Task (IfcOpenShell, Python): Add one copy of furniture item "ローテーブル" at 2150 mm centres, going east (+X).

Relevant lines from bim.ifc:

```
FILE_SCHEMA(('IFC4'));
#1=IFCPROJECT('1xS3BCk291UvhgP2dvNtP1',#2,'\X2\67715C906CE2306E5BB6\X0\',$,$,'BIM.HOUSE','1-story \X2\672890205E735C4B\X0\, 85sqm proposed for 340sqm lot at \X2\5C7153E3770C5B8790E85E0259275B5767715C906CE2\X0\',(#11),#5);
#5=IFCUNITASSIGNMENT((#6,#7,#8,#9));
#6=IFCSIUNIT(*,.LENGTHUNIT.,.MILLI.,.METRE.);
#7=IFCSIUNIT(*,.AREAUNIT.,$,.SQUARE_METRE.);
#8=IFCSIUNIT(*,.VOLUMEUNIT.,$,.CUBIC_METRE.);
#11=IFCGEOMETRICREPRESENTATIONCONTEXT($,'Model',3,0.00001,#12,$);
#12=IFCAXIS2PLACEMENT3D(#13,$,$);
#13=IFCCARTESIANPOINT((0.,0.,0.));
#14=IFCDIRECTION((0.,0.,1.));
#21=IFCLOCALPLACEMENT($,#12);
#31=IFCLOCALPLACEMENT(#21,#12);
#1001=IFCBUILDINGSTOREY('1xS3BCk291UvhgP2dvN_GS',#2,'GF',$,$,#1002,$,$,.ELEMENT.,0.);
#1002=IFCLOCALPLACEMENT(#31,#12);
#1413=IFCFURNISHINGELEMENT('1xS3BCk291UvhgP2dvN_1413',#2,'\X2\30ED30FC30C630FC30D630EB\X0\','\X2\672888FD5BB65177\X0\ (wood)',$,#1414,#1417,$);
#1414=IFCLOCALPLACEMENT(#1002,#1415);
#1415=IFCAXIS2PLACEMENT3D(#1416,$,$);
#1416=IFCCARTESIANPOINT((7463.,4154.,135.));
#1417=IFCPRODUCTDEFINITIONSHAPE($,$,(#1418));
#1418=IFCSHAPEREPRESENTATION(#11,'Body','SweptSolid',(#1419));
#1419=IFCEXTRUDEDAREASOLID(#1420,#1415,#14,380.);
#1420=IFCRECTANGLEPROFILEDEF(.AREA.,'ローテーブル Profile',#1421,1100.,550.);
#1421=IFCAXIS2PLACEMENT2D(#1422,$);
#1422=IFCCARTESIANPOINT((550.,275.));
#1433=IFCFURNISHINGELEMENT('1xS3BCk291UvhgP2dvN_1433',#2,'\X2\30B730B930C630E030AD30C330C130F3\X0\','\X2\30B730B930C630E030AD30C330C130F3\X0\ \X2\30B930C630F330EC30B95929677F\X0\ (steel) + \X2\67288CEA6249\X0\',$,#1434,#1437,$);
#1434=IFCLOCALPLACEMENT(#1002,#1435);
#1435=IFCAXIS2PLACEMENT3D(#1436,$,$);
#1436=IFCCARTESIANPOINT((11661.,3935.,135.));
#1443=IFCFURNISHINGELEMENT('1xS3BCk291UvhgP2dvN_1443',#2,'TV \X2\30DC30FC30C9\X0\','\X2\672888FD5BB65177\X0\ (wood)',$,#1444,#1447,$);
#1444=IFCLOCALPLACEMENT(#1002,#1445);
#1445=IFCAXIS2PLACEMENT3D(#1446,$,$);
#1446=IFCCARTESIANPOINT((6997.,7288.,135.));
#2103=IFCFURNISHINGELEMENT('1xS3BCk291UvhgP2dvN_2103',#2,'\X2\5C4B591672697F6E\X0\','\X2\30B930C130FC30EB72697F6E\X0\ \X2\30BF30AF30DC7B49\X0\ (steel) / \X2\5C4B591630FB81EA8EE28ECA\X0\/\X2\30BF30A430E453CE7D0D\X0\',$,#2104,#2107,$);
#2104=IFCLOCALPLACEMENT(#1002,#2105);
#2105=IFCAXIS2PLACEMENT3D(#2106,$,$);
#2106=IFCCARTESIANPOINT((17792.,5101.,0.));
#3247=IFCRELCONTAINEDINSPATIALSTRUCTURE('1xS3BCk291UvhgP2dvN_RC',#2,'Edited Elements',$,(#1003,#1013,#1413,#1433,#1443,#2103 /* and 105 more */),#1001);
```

```python
import numpy as np
import ifcopenshell
import ifcopenshell.api.geometry
import ifcopenshell.api.root
import ifcopenshell.util.element
import ifcopenshell.util.placement

model = ifcopenshell.open("bim.ifc")


def reuse_history(source, copy):
    """copy_class also copies each property set's owner history, people and application; keep the originals."""
    for rel in copy.IsDefinedBy:
        if rel.is_a("IfcRelDefinesByProperties") and (history := rel.RelatingPropertyDefinition.OwnerHistory):
            rel.RelatingPropertyDefinition.OwnerHistory = source.OwnerHistory
            ifcopenshell.util.element.remove_deep2(model, history)


source = model.by_guid("1xS3BCk291UvhgP2dvN_1413")
base = ifcopenshell.util.placement.get_local_placement(source.ObjectPlacement)
step = np.array([1.0, 0.0, 0.0]) * 2150.0

for i in range(1, 2):
    copy = ifcopenshell.api.root.copy_class(model, product=source)
    copy.Representation = ifcopenshell.util.element.copy_deep(
        model, source.Representation, exclude=["IfcGeometricRepresentationContext", "IfcRepresentationMap"]
    )
    reuse_history(source, copy)
    matrix = base.copy()
    matrix[:3, 3] += i * step
    print("added at", matrix[:3, 3].round(3) + 0.0)
    ifcopenshell.api.geometry.edit_object_placement(model, product=copy, matrix=matrix, is_si=False)

model.write("bim_updated.ifc")
```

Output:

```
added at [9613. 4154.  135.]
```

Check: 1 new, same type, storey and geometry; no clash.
